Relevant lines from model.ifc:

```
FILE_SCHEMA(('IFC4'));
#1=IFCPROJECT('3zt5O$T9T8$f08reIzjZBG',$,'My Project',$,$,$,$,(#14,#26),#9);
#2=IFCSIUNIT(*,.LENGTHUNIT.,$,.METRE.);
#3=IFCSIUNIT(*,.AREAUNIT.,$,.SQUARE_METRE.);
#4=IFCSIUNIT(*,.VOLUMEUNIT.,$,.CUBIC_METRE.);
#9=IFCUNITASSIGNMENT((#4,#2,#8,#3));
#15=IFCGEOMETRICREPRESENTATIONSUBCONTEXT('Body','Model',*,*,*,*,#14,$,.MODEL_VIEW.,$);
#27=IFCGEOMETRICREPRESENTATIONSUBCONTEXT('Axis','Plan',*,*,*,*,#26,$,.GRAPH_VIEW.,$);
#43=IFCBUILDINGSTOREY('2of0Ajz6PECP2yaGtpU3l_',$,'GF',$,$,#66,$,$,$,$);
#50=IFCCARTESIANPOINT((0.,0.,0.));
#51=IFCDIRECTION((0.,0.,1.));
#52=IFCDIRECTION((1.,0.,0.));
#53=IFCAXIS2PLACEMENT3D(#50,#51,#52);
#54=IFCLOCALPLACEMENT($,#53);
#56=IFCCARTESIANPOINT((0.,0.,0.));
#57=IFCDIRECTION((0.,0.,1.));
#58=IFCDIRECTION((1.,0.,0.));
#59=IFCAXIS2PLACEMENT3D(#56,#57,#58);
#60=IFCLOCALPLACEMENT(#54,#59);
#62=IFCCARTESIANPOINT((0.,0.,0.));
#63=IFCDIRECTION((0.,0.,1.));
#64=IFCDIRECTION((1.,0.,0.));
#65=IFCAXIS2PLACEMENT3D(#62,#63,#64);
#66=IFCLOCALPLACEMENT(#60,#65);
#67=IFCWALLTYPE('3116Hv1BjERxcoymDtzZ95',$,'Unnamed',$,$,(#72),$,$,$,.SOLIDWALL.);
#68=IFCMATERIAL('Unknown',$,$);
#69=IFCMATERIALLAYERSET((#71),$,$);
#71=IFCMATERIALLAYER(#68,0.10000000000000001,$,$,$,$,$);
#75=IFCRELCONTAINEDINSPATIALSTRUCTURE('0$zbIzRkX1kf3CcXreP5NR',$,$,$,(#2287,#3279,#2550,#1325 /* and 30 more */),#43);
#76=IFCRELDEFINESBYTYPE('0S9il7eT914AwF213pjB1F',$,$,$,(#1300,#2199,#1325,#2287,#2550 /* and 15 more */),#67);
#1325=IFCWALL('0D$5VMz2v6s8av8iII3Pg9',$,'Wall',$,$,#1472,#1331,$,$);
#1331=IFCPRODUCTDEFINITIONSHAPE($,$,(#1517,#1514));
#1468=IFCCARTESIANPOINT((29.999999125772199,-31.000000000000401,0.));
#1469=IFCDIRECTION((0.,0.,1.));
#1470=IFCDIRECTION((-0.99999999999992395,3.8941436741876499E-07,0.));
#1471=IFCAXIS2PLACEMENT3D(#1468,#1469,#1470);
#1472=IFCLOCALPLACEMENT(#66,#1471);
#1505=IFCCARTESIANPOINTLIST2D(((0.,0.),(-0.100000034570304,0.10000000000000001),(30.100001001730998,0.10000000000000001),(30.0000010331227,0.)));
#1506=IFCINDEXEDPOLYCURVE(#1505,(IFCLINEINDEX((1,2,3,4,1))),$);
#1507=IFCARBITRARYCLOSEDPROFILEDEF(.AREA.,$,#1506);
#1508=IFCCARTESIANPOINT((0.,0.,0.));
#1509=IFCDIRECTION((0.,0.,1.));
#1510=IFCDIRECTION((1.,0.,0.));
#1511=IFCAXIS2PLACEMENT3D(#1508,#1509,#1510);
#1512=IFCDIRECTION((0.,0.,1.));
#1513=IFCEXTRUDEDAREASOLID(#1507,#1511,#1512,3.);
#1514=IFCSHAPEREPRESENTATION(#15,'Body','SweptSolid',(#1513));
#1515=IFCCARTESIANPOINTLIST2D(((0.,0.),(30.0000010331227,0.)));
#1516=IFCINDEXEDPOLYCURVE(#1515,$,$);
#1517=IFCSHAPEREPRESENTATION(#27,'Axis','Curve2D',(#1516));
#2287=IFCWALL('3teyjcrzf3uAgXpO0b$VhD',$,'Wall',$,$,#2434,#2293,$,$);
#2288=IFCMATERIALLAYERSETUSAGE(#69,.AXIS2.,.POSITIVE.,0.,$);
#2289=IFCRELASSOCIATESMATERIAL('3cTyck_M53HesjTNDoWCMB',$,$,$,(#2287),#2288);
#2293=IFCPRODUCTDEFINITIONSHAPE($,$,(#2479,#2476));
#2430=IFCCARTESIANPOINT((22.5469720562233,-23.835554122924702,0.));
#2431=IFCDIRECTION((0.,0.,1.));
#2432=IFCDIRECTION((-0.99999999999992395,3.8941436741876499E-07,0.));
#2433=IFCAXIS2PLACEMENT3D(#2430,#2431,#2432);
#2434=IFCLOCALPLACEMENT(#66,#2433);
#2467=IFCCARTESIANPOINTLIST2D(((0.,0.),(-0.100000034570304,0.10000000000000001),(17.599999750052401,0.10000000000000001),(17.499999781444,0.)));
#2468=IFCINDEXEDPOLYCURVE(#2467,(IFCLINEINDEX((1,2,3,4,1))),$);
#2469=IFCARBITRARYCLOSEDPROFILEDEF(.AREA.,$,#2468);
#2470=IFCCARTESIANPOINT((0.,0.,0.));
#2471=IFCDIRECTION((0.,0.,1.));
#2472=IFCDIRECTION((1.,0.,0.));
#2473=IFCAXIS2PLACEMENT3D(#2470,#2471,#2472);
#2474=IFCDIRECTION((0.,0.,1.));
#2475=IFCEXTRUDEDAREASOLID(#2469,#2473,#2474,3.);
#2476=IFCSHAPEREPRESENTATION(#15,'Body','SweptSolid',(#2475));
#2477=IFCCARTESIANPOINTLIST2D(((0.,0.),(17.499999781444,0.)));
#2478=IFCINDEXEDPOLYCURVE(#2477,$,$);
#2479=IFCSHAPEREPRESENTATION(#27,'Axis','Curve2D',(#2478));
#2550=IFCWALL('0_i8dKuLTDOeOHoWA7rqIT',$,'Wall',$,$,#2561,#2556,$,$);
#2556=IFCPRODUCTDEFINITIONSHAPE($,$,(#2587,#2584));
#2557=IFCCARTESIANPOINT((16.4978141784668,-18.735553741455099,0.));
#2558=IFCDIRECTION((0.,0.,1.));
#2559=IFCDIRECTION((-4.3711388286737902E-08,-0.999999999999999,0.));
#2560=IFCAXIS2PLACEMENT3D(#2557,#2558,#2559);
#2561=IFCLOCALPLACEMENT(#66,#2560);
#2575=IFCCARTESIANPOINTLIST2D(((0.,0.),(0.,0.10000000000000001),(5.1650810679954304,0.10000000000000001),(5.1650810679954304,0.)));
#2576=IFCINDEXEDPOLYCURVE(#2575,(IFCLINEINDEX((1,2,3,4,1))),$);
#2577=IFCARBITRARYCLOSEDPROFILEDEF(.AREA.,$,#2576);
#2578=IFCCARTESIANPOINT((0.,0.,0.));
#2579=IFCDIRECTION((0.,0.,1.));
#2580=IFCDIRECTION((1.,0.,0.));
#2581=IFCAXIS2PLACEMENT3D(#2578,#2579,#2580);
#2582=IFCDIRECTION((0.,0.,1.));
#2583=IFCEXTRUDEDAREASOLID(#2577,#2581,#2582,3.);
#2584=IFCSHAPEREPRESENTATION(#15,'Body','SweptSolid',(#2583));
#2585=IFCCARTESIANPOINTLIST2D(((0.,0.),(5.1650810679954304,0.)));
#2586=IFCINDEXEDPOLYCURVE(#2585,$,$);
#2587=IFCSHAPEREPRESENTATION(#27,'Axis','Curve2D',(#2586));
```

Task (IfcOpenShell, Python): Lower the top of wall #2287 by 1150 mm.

```python
import ifcopenshell
import ifcopenshell.geom
import ifcopenshell.util.representation
import ifcopenshell.util.shape
import ifcopenshell.util.unit

model = ifcopenshell.open("model.ifc")
unit_scale = ifcopenshell.util.unit.calculate_unit_scale(model)
settings = ifcopenshell.geom.settings()


def volume(element):
    """Net volume in cubic metres, openings subtracted."""
    shape = ifcopenshell.geom.create_shape(settings, element)
    return ifcopenshell.util.shape.get_volume(shape.geometry)


wall = model.by_id(2287)
before = volume(wall)

body = ifcopenshell.util.representation.get_representation(wall, "Model", "Body")
solid = body.Items[0]
old_height = solid.Depth
solid.Depth -= 1.15 / unit_scale
after = volume(wall)

print(f"height {old_height:g} -> {solid.Depth:g}, volume {before:.3f} -> {after:.3f} m3")

model.write("model-out.ifc")
```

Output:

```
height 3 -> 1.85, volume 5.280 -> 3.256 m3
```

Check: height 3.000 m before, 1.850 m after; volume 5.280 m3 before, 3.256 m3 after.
